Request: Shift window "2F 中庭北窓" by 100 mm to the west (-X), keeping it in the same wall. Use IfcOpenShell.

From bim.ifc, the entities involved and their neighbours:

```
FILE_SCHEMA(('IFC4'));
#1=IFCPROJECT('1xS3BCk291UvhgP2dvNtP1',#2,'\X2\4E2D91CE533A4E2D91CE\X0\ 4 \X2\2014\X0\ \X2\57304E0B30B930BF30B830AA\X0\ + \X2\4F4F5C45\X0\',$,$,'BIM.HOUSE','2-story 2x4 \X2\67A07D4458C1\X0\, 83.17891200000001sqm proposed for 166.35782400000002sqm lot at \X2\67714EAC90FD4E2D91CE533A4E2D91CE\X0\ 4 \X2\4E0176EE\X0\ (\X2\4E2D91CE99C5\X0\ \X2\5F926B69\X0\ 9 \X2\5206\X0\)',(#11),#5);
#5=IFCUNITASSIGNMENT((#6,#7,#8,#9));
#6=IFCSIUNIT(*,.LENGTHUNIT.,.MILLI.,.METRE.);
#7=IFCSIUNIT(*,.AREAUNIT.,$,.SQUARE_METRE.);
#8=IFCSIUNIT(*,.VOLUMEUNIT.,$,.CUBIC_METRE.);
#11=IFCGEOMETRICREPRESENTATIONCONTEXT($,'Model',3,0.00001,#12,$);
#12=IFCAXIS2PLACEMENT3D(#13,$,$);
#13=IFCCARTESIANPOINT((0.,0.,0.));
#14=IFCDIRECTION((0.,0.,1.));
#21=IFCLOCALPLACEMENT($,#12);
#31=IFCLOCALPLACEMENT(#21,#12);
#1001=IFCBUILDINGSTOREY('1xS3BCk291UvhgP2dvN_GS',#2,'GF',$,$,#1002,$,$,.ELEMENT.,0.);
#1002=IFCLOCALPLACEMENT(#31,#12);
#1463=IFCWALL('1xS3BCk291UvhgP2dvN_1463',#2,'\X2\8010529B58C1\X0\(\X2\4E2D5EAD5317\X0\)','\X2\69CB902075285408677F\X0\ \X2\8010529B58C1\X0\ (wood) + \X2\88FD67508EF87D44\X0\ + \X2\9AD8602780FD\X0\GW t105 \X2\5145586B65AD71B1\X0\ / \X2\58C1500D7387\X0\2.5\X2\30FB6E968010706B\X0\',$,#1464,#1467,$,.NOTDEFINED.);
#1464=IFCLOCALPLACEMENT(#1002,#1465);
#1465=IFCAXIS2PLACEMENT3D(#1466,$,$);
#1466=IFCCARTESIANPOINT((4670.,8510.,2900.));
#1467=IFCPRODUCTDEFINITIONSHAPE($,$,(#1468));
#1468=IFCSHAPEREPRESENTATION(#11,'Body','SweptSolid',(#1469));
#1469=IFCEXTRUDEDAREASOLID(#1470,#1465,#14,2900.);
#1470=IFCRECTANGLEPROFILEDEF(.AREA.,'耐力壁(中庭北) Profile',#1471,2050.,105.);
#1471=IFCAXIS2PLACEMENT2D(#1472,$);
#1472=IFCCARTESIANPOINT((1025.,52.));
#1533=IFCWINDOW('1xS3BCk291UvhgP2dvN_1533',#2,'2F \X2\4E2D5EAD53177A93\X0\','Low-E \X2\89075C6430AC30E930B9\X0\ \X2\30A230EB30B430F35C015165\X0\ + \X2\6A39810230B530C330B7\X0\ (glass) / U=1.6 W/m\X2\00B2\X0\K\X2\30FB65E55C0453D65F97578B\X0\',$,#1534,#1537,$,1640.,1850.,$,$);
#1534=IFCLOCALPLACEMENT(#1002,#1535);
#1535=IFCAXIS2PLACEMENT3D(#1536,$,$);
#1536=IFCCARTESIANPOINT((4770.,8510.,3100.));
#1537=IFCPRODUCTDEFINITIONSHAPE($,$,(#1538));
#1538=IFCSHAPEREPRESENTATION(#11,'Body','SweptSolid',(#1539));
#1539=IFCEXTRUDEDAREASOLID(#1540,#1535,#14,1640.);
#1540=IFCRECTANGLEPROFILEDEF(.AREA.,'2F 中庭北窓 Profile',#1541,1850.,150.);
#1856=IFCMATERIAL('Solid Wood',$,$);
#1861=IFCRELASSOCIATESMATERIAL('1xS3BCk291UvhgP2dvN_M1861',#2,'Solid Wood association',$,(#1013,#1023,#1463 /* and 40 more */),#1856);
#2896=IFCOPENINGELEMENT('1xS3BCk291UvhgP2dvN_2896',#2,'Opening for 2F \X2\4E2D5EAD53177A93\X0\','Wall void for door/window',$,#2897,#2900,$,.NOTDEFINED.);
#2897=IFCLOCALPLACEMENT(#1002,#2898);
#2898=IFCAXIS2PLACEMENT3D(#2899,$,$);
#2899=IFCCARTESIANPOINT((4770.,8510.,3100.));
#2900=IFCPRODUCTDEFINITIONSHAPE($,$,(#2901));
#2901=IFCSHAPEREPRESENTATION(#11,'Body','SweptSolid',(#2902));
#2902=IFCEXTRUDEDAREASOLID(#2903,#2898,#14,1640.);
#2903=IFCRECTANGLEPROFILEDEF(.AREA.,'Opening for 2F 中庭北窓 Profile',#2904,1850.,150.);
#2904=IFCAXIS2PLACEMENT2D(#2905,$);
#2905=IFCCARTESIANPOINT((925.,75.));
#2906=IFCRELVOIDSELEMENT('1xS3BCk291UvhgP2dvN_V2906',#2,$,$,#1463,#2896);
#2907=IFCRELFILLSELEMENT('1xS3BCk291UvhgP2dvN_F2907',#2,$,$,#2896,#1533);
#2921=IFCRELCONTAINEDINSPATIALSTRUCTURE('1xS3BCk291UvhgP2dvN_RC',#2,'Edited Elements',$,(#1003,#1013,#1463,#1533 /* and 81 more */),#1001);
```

```python
import ifcopenshell
import ifcopenshell.api.geometry
import ifcopenshell.util.placement
import ifcopenshell.util.unit

model = ifcopenshell.open("bim.ifc")
unit_scale = ifcopenshell.util.unit.calculate_unit_scale(model)

window = model.by_id(1533)
opening = window.FillsVoids[0].RelatingOpeningElement
wall = opening.VoidsElements[0].RelatingBuildingElement

wall_matrix = ifcopenshell.util.placement.get_local_placement(wall.ObjectPlacement)
shift = wall_matrix[:3, 0] * -0.1 / unit_scale
before = ifcopenshell.util.placement.get_local_placement(window.ObjectPlacement)[:3, 3].copy()

# The window is not placed relative to its opening, so move both.
for product in (opening, window):
    matrix = ifcopenshell.util.placement.get_local_placement(product.ObjectPlacement)
    matrix[:3, 3] += shift
    ifcopenshell.api.geometry.edit_object_placement(model, product=product, matrix=matrix, is_si=False)

after = ifcopenshell.util.placement.get_local_placement(window.ObjectPlacement)[:3, 3]
print("window moved by", (after - before).round(3) + 0.0)

model.write("bim_v2.ifc")
```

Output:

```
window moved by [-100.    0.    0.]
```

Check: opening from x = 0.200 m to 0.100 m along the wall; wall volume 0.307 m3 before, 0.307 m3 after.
